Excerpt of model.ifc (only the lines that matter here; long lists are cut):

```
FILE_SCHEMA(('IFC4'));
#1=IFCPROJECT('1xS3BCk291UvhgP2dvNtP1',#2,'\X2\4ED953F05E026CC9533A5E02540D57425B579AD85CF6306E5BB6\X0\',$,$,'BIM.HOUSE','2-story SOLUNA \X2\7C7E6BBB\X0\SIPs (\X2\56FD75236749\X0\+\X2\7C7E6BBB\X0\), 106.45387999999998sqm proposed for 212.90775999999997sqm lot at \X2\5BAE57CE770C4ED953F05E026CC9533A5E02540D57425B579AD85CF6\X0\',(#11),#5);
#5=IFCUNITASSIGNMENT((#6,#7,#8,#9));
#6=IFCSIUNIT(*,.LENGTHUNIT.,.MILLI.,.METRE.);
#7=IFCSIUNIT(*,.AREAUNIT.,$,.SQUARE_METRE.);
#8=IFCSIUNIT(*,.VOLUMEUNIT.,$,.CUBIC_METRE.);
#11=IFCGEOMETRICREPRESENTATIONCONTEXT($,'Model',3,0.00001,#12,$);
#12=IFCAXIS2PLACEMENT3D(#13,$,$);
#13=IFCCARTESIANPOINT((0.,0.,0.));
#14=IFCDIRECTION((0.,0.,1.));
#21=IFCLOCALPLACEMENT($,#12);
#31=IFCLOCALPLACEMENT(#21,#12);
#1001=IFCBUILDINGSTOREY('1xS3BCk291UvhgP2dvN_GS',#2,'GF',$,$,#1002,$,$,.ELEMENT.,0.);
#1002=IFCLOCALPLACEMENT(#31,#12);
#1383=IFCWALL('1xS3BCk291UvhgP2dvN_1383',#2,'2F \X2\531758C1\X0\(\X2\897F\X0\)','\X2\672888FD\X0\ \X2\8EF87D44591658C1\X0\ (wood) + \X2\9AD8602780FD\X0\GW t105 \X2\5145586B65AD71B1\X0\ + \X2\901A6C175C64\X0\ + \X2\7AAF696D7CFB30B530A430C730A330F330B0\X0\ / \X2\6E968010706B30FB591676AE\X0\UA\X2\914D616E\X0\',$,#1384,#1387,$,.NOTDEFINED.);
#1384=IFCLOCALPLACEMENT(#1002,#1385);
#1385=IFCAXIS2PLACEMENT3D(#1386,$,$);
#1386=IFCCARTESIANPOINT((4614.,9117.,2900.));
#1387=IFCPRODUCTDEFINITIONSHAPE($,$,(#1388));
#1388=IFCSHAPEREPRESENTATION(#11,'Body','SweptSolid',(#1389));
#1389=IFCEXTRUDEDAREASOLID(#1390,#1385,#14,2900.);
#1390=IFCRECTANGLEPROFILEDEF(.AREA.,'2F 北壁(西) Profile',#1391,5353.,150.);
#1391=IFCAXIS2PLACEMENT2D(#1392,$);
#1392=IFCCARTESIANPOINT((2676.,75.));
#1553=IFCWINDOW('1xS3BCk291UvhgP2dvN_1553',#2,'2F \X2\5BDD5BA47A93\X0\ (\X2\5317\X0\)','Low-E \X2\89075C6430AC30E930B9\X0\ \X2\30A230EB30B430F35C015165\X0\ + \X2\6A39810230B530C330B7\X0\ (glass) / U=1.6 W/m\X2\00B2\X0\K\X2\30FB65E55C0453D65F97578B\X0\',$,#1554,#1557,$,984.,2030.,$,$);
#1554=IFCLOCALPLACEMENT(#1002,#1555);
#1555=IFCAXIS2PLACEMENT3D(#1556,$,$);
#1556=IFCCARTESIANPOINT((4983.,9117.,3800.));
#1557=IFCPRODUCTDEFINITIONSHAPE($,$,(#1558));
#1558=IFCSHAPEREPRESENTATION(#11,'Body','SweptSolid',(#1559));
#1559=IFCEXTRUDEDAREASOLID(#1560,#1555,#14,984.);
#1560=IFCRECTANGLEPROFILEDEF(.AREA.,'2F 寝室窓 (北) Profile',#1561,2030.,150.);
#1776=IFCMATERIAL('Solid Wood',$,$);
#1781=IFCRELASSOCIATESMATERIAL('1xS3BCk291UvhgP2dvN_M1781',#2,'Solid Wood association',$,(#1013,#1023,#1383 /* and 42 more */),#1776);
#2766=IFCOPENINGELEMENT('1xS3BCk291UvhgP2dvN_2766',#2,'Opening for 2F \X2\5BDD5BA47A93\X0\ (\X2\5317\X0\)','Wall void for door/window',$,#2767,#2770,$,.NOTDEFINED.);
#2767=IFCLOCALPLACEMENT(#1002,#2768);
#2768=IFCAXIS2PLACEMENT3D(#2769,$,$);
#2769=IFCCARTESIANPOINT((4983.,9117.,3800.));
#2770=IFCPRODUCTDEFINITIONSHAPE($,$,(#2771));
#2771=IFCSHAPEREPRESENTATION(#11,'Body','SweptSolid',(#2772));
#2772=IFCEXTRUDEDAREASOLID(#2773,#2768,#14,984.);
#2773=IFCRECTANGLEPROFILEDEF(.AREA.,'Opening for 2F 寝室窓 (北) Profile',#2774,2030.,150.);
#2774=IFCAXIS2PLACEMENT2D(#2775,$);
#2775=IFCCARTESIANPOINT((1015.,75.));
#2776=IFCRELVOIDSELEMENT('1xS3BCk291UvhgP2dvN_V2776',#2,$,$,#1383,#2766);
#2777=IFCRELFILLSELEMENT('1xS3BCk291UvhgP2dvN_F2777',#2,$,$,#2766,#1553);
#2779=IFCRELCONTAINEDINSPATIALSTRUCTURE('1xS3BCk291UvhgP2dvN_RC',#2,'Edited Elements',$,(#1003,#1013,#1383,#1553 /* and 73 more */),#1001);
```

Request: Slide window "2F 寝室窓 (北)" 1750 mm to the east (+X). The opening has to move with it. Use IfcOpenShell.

```python
import ifcopenshell
import ifcopenshell.api.geometry
import ifcopenshell.util.placement
import ifcopenshell.util.unit

model = ifcopenshell.open("model.ifc")
unit_scale = ifcopenshell.util.unit.calculate_unit_scale(model)

window = model.by_guid("1xS3BCk291UvhgP2dvN_1553")
opening = window.FillsVoids[0].RelatingOpeningElement
wall = opening.VoidsElements[0].RelatingBuildingElement

wall_matrix = ifcopenshell.util.placement.get_local_placement(wall.ObjectPlacement)
shift = wall_matrix[:3, 0] * 1.75 / unit_scale
before = ifcopenshell.util.placement.get_local_placement(window.ObjectPlacement)[:3, 3].copy()

# The window is not placed relative to its opening, so move both.
for product in (opening, window):
    matrix = ifcopenshell.util.placement.get_local_placement(product.ObjectPlacement)
    matrix[:3, 3] += shift
    ifcopenshell.api.geometry.edit_object_placement(model, product=product, matrix=matrix, is_si=False)

after = ifcopenshell.util.placement.get_local_placement(window.ObjectPlacement)[:3, 3]
print("window moved by", (after - before).round(3) + 0.0)

model.write("model_rev.ifc")
```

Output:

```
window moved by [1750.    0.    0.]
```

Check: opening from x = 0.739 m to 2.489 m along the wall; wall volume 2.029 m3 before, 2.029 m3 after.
